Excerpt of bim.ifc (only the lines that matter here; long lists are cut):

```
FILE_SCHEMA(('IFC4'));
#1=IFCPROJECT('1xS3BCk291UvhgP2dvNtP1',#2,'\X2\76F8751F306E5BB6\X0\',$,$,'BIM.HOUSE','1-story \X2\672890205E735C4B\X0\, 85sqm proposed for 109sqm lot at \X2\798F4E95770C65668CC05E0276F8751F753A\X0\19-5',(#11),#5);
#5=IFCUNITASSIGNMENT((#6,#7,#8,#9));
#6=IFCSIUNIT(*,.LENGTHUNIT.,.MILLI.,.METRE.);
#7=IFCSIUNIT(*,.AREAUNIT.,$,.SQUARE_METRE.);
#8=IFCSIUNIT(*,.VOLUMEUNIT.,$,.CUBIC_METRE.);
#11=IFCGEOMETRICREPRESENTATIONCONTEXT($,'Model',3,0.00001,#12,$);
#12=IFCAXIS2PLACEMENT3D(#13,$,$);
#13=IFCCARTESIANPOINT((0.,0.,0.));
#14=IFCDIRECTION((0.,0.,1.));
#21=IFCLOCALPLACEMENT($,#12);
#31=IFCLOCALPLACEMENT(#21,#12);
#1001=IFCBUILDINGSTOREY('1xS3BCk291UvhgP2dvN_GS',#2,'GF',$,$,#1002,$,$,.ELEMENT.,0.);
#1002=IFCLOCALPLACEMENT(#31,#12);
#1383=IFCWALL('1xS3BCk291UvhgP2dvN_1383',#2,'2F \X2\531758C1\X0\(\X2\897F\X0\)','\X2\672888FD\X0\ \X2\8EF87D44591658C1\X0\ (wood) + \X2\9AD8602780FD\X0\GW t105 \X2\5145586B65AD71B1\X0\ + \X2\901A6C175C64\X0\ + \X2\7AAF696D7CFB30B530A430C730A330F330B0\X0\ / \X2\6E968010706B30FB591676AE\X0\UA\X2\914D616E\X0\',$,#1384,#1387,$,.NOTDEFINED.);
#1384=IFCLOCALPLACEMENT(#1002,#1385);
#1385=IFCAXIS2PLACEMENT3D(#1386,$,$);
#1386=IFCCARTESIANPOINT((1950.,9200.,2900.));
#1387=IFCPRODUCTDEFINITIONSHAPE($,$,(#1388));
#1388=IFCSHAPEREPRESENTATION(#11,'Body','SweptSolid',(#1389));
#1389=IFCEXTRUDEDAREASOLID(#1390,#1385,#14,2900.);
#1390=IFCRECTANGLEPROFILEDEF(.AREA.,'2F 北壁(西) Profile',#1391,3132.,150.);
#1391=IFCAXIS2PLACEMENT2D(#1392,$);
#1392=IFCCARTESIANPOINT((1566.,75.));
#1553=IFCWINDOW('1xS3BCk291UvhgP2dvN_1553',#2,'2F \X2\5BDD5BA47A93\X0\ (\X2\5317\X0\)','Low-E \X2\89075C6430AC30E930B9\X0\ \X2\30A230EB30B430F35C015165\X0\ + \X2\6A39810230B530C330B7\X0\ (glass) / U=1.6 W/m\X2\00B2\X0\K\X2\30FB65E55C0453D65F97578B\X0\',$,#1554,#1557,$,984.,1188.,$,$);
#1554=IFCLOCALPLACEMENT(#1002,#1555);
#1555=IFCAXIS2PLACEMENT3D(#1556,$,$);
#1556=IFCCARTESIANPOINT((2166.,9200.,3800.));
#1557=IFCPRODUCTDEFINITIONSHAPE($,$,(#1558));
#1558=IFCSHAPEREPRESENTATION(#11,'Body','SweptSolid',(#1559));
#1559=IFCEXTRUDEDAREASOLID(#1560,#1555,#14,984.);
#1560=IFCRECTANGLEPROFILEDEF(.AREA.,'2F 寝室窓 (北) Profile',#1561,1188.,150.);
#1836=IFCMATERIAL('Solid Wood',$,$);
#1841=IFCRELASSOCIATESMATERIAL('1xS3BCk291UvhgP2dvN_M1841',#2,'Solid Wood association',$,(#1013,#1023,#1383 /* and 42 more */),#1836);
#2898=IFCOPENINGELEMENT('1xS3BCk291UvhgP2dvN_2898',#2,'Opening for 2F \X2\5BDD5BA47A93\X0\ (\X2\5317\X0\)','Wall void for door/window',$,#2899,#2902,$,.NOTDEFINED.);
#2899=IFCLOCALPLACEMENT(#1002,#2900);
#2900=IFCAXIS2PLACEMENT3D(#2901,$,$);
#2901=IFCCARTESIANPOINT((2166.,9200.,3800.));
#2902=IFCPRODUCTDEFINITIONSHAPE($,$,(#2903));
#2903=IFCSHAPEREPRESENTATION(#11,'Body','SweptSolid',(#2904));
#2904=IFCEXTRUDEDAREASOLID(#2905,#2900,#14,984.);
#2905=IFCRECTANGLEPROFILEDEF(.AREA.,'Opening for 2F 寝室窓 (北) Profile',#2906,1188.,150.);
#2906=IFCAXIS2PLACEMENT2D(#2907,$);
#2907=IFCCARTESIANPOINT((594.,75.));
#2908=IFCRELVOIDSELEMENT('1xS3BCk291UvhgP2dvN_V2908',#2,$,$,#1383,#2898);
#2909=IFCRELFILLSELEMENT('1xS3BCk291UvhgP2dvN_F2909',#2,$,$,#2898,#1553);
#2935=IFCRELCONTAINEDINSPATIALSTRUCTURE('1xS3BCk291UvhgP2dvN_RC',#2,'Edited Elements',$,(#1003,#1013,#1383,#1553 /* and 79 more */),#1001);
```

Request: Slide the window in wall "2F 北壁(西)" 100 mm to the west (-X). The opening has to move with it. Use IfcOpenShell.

```python
import ifcopenshell
import ifcopenshell.api.geometry
import ifcopenshell.util.placement
import ifcopenshell.util.unit

model = ifcopenshell.open("bim.ifc")
unit_scale = ifcopenshell.util.unit.calculate_unit_scale(model)

window = model.by_guid("1xS3BCk291UvhgP2dvN_1553")
opening = window.FillsVoids[0].RelatingOpeningElement
wall = opening.VoidsElements[0].RelatingBuildingElement

wall_matrix = ifcopenshell.util.placement.get_local_placement(wall.ObjectPlacement)
shift = wall_matrix[:3, 0] * -0.1 / unit_scale
before = ifcopenshell.util.placement.get_local_placement(window.ObjectPlacement)[:3, 3].copy()

# The window is not placed relative to its opening, so move both.
for product in (opening, window):
    matrix = ifcopenshell.util.placement.get_local_placement(product.ObjectPlacement)
    matrix[:3, 3] += shift
    ifcopenshell.api.geometry.edit_object_placement(model, product=product, matrix=matrix, is_si=False)

after = ifcopenshell.util.placement.get_local_placement(window.ObjectPlacement)[:3, 3]
print("window moved by", (after - before).round(3) + 0.0)

model.write("bim_updated.ifc")
```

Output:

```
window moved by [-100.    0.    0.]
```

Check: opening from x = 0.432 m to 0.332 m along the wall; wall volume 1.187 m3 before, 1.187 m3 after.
